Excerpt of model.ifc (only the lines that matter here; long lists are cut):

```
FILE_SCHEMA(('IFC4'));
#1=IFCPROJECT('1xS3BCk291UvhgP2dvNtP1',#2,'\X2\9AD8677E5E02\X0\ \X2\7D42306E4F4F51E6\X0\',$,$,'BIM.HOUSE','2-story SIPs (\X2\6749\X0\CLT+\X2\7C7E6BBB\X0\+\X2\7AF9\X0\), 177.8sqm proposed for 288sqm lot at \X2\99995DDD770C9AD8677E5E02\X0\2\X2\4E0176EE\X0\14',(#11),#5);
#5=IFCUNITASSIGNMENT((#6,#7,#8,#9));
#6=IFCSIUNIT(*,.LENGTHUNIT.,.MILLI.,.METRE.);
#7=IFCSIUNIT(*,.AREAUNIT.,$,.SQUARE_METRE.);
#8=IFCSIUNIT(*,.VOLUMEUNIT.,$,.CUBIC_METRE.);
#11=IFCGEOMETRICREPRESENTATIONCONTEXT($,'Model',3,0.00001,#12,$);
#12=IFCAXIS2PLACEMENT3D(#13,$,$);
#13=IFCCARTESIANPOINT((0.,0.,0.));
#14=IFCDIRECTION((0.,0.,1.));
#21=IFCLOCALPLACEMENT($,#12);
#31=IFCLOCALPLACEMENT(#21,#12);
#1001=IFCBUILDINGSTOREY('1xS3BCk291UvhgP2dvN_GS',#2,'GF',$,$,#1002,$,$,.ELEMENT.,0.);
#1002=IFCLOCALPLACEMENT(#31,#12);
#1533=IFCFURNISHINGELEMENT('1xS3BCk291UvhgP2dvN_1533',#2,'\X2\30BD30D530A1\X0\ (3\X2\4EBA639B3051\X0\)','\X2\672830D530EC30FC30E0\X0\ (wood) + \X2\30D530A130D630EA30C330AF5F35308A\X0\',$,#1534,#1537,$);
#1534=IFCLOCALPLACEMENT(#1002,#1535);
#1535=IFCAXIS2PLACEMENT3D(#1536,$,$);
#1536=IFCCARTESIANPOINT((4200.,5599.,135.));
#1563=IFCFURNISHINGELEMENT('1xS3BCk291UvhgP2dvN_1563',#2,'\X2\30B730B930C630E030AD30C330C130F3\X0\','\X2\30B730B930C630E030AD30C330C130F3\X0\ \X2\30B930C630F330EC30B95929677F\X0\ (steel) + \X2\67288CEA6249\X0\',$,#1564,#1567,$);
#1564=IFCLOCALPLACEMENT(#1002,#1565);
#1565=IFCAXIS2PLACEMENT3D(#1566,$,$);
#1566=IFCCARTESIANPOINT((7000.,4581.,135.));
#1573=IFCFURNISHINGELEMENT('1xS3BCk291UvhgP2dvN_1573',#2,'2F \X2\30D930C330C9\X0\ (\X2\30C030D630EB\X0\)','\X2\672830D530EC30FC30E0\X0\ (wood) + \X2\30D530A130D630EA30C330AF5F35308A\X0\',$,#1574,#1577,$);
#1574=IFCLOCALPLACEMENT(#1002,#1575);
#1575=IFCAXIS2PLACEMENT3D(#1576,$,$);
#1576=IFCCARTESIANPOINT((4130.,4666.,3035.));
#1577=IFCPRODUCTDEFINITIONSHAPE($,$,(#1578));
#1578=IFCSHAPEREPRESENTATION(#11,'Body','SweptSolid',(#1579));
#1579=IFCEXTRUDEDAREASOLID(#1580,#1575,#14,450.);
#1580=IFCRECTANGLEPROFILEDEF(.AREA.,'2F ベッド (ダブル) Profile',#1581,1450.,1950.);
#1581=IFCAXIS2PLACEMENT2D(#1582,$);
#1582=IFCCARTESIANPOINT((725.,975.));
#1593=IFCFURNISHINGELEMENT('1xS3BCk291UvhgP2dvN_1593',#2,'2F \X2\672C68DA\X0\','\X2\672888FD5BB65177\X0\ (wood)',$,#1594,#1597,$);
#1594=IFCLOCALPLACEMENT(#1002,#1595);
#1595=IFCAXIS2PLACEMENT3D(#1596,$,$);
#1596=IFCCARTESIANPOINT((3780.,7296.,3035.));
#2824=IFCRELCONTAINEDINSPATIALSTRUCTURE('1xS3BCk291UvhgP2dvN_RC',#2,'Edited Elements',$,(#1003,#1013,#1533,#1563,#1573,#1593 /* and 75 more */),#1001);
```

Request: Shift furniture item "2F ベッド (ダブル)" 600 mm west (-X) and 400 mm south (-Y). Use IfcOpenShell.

```python
import ifcopenshell
import ifcopenshell.api.geometry
import ifcopenshell.util.placement

model = ifcopenshell.open("model.ifc")

item = model.by_id(1573)
matrix = ifcopenshell.util.placement.get_local_placement(item.ObjectPlacement)
matrix[0, 3] -= 600.0
matrix[1, 3] -= 400.0
ifcopenshell.api.geometry.edit_object_placement(model, product=item, matrix=matrix, is_si=False)

print(ifcopenshell.util.placement.get_local_placement(item.ObjectPlacement).round(3) + 0.0)

model.write("model_v2.ifc")
```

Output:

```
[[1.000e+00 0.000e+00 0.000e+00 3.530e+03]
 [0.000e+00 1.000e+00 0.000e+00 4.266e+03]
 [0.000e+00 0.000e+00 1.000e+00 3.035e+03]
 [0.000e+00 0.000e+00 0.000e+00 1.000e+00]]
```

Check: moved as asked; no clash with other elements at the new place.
